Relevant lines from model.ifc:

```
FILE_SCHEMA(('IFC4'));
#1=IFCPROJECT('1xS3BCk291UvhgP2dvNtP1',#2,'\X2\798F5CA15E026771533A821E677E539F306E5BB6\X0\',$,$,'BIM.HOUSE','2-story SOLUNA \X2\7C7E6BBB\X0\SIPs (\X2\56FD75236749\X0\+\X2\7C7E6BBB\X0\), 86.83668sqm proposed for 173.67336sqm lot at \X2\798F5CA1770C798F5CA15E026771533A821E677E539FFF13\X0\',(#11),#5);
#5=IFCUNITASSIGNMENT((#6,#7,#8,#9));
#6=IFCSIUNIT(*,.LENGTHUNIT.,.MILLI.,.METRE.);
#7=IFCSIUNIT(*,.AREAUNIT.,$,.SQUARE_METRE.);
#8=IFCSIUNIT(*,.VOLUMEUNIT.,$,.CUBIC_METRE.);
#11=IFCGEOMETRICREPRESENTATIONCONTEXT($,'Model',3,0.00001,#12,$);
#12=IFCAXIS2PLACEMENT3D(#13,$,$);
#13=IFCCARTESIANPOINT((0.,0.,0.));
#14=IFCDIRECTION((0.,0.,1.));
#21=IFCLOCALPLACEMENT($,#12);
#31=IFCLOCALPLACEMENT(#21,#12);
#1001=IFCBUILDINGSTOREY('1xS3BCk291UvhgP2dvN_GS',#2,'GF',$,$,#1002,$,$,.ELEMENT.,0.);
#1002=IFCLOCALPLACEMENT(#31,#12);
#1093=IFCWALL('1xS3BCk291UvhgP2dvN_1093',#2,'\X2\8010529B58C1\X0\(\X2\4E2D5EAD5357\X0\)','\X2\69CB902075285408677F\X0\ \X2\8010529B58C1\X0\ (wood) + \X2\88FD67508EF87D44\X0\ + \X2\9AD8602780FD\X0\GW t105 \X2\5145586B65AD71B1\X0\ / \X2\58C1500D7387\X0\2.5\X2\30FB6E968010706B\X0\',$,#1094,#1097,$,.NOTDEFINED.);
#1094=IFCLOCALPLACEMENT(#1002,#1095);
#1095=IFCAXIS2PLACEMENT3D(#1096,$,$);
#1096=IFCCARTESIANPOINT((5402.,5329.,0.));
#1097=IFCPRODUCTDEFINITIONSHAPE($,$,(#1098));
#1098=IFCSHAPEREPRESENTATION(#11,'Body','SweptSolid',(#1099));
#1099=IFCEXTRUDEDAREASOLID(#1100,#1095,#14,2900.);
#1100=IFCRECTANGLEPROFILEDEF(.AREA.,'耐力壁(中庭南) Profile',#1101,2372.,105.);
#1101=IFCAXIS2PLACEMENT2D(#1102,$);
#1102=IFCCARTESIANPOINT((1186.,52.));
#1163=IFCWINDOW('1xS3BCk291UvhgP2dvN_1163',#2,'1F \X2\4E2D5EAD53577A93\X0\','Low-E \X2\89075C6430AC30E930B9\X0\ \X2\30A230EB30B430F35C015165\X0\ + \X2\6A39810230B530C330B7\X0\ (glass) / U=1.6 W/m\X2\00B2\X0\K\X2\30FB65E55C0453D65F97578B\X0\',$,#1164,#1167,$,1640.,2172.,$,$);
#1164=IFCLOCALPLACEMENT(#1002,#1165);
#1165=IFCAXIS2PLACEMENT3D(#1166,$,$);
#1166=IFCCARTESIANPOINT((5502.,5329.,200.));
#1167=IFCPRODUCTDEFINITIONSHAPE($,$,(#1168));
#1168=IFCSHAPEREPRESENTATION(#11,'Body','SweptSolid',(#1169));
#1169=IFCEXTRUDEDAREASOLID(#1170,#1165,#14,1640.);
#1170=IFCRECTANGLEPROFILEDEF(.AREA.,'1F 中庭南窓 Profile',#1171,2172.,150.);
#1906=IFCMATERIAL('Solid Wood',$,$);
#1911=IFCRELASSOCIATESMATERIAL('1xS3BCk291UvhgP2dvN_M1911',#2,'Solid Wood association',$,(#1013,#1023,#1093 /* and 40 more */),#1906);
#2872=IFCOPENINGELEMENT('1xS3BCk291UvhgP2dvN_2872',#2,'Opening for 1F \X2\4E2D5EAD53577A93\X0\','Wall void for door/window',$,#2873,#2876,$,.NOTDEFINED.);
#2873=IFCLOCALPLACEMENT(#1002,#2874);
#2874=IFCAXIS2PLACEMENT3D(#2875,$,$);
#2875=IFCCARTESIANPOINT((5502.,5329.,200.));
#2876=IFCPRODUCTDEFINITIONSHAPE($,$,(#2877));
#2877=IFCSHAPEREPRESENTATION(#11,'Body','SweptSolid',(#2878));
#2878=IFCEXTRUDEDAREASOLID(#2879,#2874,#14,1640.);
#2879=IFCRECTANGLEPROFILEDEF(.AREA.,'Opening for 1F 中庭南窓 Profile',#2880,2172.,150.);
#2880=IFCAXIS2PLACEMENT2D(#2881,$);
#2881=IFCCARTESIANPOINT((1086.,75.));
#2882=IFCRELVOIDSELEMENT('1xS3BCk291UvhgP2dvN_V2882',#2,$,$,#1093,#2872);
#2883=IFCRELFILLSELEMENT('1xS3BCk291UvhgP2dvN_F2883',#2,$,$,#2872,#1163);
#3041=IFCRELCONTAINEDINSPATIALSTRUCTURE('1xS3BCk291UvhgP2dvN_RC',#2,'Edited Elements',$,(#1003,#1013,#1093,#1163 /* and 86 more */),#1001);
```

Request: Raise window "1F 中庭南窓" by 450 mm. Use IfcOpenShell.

```python
import numpy as np
import ifcopenshell
import ifcopenshell.api.geometry
import ifcopenshell.util.placement
import ifcopenshell.util.unit

model = ifcopenshell.open("model.ifc")
unit_scale = ifcopenshell.util.unit.calculate_unit_scale(model)

window = model.by_id(1163)
opening = window.FillsVoids[0].RelatingOpeningElement
dz = 0.45 / unit_scale

shift = np.array([0.0, 0.0, dz])
# The window is not placed relative to its opening, so move both.
for product in (opening, window):
    matrix = ifcopenshell.util.placement.get_local_placement(product.ObjectPlacement)
    matrix[:3, 3] += shift
    ifcopenshell.api.geometry.edit_object_placement(model, product=product, matrix=matrix, is_si=False)

print(f"moved by {dz * unit_scale:+.3f} m")

model.write("model_v2.ifc")
```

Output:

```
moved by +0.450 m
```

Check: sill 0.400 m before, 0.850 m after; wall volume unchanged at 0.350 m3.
